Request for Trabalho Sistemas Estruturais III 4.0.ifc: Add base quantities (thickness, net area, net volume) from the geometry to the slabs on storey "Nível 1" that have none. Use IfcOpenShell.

First a look at what the model holds.

```python
import ifcopenshell
import ifcopenshell.util.element
import ifcopenshell.util.unit

model = ifcopenshell.open("Trabalho Sistemas Estruturais III 4.0.ifc")
print(model.schema)
for unit_type in ("LENGTHUNIT", "AREAUNIT", "VOLUMEUNIT"):
    print(unit_type, ifcopenshell.util.unit.calculate_unit_scale(model, unit_type))
storey = next(s for s in model.by_type("IfcBuildingStorey") if s.Name == "Nível 1")
slabs = [e for e in ifcopenshell.util.element.get_decomposition(storey) if e.is_a("IfcSlab")]
for e in sorted(slabs, key=lambda e: e.id()):
    print(e.id(), e.is_a(), e.Name, list(ifcopenshell.util.element.get_psets(e, qtos_only=True)), sep=" | ")
```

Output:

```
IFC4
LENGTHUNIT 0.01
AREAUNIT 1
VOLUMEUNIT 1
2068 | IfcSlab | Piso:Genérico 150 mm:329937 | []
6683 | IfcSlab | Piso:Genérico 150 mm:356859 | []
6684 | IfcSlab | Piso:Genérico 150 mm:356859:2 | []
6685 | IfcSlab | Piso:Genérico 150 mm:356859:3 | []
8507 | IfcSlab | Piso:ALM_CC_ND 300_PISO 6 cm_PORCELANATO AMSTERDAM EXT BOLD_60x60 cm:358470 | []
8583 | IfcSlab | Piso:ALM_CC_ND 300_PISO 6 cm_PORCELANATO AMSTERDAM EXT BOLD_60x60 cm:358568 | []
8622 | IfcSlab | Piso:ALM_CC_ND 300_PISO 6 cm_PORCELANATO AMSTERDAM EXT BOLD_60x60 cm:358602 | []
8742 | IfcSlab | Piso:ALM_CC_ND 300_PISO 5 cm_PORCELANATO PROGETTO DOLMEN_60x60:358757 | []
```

```python
import ifcopenshell
import ifcopenshell.api.pset
import ifcopenshell.geom
import ifcopenshell.util.element
import ifcopenshell.util.shape
import ifcopenshell.util.unit

model = ifcopenshell.open("Trabalho Sistemas Estruturais III 4.0.ifc")
unit_scale = ifcopenshell.util.unit.calculate_unit_scale(model)
area_scale = ifcopenshell.util.unit.calculate_unit_scale(model, "AREAUNIT")
volume_scale = ifcopenshell.util.unit.calculate_unit_scale(model, "VOLUMEUNIT")
settings = ifcopenshell.geom.settings()

storey = next(s for s in model.by_type("IfcBuildingStorey") if s.Name == "Nível 1")
slabs = [e for e in ifcopenshell.util.element.get_decomposition(storey) if e.is_a("IfcSlab")]

for e in sorted(slabs, key=lambda e: e.id()):
    if ifcopenshell.util.element.get_psets(e, qtos_only=True, should_inherit=False):
        continue
    # Geometry comes back in metres, in the element's own axes.
    shape = ifcopenshell.geom.create_shape(settings, e)
    values = {
        "Width": ifcopenshell.util.shape.get_z(shape.geometry) / unit_scale,
        "NetArea": ifcopenshell.util.shape.get_footprint_area(shape.geometry) / area_scale,
        "NetVolume": ifcopenshell.util.shape.get_volume(shape.geometry) / volume_scale,
    }
    qto = ifcopenshell.api.pset.add_qto(model, product=e, name="Qto_SlabBaseQuantities")
    ifcopenshell.api.pset.edit_qto(model, qto=qto, properties=values)
    print(e.id(), {k: round(v, 3) for k, v in values.items()})

model.write("Trabalho Sistemas Estruturais III 4.0_v2.ifc")
```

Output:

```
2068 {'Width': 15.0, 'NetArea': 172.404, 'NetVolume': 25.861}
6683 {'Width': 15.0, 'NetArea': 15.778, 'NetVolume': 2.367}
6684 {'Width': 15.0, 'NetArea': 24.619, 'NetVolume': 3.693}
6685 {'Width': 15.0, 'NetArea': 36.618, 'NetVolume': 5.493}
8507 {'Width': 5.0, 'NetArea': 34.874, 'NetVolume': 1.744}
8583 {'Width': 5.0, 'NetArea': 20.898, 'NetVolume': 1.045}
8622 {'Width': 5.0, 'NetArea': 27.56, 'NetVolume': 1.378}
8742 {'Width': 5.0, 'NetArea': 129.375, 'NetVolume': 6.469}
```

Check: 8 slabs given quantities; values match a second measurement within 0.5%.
